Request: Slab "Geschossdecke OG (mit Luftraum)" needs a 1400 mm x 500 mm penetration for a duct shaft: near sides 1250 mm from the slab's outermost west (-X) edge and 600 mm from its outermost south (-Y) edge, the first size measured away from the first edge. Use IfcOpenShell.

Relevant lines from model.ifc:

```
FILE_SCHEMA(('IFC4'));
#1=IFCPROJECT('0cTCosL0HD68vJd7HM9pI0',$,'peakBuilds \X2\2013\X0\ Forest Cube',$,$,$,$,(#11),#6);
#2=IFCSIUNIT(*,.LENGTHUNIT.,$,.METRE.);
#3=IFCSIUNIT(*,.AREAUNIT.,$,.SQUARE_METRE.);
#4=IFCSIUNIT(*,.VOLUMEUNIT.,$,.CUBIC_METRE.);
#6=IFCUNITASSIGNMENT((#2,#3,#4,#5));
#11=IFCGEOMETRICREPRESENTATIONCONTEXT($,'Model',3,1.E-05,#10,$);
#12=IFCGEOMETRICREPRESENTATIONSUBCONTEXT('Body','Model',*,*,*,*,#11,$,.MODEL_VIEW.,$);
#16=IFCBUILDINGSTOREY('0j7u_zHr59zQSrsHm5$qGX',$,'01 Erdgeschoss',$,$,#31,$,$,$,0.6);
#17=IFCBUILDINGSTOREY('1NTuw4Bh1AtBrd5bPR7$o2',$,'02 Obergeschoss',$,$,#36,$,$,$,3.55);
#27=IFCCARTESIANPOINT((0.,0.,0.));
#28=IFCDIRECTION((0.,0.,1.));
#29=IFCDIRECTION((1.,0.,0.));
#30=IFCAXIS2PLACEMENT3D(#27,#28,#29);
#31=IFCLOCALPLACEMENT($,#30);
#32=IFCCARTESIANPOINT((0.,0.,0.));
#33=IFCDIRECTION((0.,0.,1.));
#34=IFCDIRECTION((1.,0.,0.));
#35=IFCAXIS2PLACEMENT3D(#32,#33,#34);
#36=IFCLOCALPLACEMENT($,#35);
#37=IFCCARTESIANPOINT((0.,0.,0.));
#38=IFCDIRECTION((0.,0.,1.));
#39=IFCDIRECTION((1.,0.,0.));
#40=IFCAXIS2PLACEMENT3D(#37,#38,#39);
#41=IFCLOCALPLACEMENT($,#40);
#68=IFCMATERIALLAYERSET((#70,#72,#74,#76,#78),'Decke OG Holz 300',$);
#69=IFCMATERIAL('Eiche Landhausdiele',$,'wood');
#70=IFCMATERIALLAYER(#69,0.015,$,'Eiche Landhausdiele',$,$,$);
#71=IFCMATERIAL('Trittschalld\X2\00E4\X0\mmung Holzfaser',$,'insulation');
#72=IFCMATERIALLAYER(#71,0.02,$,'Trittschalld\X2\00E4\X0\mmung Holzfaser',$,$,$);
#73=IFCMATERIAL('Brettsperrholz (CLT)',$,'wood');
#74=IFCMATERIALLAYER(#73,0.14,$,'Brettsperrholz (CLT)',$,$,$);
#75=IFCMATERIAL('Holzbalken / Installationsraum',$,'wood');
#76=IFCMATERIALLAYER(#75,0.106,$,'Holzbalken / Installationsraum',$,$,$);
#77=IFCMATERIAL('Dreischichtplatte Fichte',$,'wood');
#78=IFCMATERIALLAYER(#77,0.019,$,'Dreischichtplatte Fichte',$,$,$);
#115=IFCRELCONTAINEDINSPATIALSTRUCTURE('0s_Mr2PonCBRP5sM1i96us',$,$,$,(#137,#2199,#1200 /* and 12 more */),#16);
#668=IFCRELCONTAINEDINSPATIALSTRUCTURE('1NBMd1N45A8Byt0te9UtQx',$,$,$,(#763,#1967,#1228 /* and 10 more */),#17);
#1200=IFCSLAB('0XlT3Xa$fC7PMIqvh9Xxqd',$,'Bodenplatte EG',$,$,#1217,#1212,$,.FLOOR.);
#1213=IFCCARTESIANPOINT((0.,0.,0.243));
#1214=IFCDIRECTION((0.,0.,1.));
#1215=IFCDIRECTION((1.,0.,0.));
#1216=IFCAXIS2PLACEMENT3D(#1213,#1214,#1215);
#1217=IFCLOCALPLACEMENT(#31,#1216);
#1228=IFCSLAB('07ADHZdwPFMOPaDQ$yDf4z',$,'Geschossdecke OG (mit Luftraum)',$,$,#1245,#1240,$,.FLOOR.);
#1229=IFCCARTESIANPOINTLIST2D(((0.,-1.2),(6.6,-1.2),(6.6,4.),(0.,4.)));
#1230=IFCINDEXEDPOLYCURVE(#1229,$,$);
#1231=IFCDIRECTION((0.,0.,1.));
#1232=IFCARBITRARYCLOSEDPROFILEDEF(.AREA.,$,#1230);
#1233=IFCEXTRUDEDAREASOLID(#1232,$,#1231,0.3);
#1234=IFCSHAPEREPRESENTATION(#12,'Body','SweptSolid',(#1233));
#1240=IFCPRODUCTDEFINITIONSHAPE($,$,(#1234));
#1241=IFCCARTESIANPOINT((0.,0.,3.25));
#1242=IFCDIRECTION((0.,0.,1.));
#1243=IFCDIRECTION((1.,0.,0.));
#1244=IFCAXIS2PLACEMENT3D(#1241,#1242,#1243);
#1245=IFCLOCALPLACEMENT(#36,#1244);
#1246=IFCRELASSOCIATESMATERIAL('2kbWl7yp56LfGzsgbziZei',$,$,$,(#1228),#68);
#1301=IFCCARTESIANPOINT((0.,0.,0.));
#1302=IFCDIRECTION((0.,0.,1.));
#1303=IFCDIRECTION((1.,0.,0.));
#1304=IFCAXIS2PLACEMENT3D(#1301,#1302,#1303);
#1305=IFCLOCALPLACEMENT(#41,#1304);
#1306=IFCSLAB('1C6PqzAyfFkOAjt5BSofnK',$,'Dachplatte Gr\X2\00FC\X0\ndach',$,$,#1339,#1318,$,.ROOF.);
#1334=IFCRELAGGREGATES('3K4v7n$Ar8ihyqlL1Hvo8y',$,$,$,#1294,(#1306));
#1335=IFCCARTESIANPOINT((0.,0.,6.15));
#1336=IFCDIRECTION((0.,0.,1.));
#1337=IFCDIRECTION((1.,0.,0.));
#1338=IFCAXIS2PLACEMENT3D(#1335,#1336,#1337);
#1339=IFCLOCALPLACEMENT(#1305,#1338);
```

```python
import numpy as np
import ifcopenshell
import ifcopenshell.api.feature
import ifcopenshell.api.geometry
import ifcopenshell.api.root
import ifcopenshell.geom
import ifcopenshell.util.placement
import ifcopenshell.util.representation
import ifcopenshell.util.shape
import ifcopenshell.util.unit

model = ifcopenshell.open("model.ifc")
unit_scale = ifcopenshell.util.unit.calculate_unit_scale(model)
settings = ifcopenshell.geom.settings()


def volume(element):
    """Net volume in cubic metres, openings subtracted."""
    shape = ifcopenshell.geom.create_shape(settings, element)
    return ifcopenshell.util.shape.get_volume(shape.geometry)


slab = model.by_guid("07ADHZdwPFMOPaDQ$yDf4z")
before = volume(slab)

# Extent in the slab's own axes, in metres. The edges named are its -X and -Y sides.
slab_shape = ifcopenshell.geom.create_shape(settings, slab)
vertices = ifcopenshell.util.shape.get_vertices(slab_shape.geometry)
x_min, y_min, bottom = vertices.min(axis=0)
top = vertices[:, 2].max()

opening = ifcopenshell.api.root.create_entity(model, ifc_class="IfcOpeningElement", name="Duct shaft opening", predefined_type="OPENING")
context = ifcopenshell.util.representation.get_context(model, "Model", "Body", "MODEL_VIEW")
width, depth = 1.4, 0.5
outline = [(0.0, 0.0), (width, 0.0), (width, depth), (0.0, depth), (0.0, 0.0)]
# Overshoot both faces by 50 mm so the cut is clean.
shape = ifcopenshell.api.geometry.add_slab_representation(
    model, context=context, depth=top - bottom + 0.1, polyline=outline
)
ifcopenshell.api.geometry.assign_representation(model, product=opening, representation=shape)

matrix = ifcopenshell.util.placement.get_local_placement(slab.ObjectPlacement)
matrix[:, 3] = matrix @ np.append(np.array([x_min + 1.25, y_min + 0.6, bottom - 0.05]) / unit_scale, 1.0)
ifcopenshell.api.geometry.edit_object_placement(model, product=opening, matrix=matrix, is_si=False)
ifcopenshell.api.feature.add_feature(model, feature=opening, element=slab)

after = volume(slab)

print(f"slab volume {before:.3f} -> {after:.3f} m3")

model.write("model-out.ifc")
```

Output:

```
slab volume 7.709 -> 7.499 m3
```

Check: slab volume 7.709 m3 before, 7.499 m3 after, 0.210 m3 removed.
